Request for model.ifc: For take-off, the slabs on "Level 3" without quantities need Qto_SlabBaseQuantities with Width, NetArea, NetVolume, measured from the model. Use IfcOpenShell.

First a look at what the model holds.

```python
import ifcopenshell
import ifcopenshell.util.element
import ifcopenshell.util.unit

model = ifcopenshell.open("model.ifc")
print(model.schema)
for unit_type in ("LENGTHUNIT", "AREAUNIT", "VOLUMEUNIT"):
    print(unit_type, ifcopenshell.util.unit.calculate_unit_scale(model, unit_type))
storey = next(s for s in model.by_type("IfcBuildingStorey") if s.Name == "Level 3")
slabs = [e for e in ifcopenshell.util.element.get_decomposition(storey) if e.is_a("IfcSlab")]
for e in sorted(slabs, key=lambda e: e.id()):
    print(e.id(), e.is_a(), e.Name, list(ifcopenshell.util.element.get_psets(e, qtos_only=True)), sep=" | ")
```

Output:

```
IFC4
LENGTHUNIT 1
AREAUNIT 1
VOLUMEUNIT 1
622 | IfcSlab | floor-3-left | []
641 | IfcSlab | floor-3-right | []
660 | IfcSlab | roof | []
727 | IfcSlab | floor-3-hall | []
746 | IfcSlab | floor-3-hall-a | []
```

```python
import ifcopenshell
import ifcopenshell.api.pset
import ifcopenshell.geom
import ifcopenshell.util.element
import ifcopenshell.util.shape
import ifcopenshell.util.unit

model = ifcopenshell.open("model.ifc")
unit_scale = ifcopenshell.util.unit.calculate_unit_scale(model)
area_scale = ifcopenshell.util.unit.calculate_unit_scale(model, "AREAUNIT")
volume_scale = ifcopenshell.util.unit.calculate_unit_scale(model, "VOLUMEUNIT")
settings = ifcopenshell.geom.settings()

storey = next(s for s in model.by_type("IfcBuildingStorey") if s.Name == "Level 3")
slabs = [e for e in ifcopenshell.util.element.get_decomposition(storey) if e.is_a("IfcSlab")]

for e in sorted(slabs, key=lambda e: e.id()):
    if ifcopenshell.util.element.get_psets(e, qtos_only=True, should_inherit=False):
        continue
    # Geometry comes back in metres, in the element's own axes.
    shape = ifcopenshell.geom.create_shape(settings, e)
    values = {
        "Width": ifcopenshell.util.shape.get_z(shape.geometry) / unit_scale,
        "NetArea": ifcopenshell.util.shape.get_footprint_area(shape.geometry) / area_scale,
        "NetVolume": ifcopenshell.util.shape.get_volume(shape.geometry) / volume_scale,
    }
    qto = ifcopenshell.api.pset.add_qto(model, product=e, name="Qto_SlabBaseQuantities")
    ifcopenshell.api.pset.edit_qto(model, qto=qto, properties=values)
    print(e.id(), {k: round(v, 3) for k, v in values.items()})

model.write("model_updated.ifc")
```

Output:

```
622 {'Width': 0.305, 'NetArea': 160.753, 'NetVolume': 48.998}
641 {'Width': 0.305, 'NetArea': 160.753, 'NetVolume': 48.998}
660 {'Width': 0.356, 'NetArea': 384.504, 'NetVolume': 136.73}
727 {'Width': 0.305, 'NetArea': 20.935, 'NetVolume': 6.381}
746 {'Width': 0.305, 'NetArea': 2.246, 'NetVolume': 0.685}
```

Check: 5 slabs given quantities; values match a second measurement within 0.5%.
